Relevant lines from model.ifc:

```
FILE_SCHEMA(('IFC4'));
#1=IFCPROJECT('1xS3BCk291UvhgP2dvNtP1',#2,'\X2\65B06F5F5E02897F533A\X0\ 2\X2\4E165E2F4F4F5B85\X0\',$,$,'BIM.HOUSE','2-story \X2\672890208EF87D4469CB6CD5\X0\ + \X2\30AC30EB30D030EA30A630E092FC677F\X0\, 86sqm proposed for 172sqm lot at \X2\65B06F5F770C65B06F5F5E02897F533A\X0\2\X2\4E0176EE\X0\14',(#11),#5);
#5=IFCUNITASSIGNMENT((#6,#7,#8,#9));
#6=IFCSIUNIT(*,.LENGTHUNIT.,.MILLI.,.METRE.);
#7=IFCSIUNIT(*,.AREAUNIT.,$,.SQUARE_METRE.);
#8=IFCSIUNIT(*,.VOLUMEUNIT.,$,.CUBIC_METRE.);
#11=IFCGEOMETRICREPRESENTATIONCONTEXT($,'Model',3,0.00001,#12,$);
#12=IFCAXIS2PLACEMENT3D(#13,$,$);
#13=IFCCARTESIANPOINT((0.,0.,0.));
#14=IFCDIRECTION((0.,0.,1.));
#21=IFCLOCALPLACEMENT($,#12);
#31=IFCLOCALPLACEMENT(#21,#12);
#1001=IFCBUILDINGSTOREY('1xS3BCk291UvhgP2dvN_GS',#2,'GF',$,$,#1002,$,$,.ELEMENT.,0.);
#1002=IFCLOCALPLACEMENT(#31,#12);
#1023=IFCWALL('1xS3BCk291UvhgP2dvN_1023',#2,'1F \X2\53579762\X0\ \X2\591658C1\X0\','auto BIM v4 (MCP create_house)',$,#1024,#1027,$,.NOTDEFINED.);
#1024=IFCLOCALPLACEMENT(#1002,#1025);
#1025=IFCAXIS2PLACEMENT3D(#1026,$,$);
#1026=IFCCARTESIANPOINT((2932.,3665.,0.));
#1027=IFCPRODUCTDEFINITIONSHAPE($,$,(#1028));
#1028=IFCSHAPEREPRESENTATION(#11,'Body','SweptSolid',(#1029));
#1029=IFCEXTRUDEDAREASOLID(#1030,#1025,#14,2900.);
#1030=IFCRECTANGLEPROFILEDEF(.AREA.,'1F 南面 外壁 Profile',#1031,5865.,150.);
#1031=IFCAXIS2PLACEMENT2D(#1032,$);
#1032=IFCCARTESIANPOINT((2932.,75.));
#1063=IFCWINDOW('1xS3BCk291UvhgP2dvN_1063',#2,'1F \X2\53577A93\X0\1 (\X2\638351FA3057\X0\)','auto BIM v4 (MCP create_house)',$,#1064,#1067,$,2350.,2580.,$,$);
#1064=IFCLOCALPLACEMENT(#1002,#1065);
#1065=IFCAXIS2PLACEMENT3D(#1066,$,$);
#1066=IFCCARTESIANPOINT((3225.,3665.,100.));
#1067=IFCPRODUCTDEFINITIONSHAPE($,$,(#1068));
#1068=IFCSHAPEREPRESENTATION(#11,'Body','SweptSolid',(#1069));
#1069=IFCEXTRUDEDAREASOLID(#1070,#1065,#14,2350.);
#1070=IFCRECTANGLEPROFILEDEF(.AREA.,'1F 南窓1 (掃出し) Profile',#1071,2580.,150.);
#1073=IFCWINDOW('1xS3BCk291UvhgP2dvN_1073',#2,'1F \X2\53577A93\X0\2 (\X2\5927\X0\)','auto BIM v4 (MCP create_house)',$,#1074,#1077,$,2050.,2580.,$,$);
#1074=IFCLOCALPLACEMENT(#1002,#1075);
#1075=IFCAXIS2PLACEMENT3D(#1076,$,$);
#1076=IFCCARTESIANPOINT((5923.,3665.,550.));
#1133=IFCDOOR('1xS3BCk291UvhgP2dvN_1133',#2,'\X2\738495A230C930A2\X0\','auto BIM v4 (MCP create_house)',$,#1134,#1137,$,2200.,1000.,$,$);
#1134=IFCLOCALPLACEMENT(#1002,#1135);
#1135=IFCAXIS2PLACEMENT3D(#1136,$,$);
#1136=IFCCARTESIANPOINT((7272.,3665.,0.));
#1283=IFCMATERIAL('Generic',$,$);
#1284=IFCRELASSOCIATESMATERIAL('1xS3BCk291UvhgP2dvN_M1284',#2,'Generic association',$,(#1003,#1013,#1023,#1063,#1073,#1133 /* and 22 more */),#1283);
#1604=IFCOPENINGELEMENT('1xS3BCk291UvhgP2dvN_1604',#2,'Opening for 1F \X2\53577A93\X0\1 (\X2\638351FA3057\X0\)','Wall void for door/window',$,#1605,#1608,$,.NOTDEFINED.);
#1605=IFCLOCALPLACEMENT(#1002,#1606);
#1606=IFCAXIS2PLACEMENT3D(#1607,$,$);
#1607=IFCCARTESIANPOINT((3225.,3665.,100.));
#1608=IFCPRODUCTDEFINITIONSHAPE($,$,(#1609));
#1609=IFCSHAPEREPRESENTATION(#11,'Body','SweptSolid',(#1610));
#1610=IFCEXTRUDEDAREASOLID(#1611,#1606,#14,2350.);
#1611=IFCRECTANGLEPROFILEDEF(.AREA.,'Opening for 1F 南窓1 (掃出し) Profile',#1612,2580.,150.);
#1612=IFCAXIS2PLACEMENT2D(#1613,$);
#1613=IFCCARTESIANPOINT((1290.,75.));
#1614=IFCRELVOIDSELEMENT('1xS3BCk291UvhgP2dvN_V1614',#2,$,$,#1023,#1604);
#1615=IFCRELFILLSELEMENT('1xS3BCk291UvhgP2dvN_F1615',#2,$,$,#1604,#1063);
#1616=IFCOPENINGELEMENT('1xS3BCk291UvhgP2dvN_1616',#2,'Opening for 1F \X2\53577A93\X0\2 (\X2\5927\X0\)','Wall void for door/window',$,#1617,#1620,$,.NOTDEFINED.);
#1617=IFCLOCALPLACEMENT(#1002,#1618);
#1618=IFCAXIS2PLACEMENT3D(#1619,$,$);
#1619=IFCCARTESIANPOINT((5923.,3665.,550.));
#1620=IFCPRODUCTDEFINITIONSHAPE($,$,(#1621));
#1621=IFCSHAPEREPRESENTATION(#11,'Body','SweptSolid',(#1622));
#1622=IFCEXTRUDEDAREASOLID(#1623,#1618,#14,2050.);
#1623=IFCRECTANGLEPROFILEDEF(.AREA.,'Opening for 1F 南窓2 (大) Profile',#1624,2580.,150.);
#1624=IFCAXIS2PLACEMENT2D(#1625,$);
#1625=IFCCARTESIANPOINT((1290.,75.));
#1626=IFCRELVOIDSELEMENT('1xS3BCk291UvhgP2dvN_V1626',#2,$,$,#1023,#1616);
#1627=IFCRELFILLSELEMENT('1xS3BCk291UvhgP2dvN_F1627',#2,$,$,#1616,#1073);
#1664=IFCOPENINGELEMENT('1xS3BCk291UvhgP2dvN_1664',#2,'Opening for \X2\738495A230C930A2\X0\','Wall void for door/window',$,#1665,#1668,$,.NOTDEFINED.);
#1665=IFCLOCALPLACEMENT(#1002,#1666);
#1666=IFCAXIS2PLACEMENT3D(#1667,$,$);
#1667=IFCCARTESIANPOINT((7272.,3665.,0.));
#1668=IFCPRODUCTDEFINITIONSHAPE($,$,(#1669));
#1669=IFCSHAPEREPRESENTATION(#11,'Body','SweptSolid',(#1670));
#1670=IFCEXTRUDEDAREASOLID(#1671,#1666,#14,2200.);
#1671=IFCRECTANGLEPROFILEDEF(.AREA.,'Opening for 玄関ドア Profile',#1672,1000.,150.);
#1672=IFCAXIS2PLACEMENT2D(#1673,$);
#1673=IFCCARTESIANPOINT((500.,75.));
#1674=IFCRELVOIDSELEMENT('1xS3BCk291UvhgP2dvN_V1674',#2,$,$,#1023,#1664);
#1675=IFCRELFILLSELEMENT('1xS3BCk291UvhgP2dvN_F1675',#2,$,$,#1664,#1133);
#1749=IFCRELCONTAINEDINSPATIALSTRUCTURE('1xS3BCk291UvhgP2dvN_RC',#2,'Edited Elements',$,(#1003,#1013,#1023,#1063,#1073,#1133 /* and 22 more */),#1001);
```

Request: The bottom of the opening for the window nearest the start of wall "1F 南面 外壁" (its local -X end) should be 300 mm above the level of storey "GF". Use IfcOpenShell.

```python
import numpy as np
import ifcopenshell
import ifcopenshell.api.geometry
import ifcopenshell.geom
import ifcopenshell.util.element
import ifcopenshell.util.placement
import ifcopenshell.util.shape
import ifcopenshell.util.unit

model = ifcopenshell.open("model.ifc")
unit_scale = ifcopenshell.util.unit.calculate_unit_scale(model)

window = model.by_guid("1xS3BCk291UvhgP2dvN_1063")
opening = window.FillsVoids[0].RelatingOpeningElement
storey = ifcopenshell.util.element.get_container(window, ifc_class="IfcBuildingStorey")
level = ifcopenshell.util.placement.get_local_placement(storey.ObjectPlacement)[2, 3]

# The opening's origin need not be at the sill, so measure its lowest point.
shape = ifcopenshell.geom.create_shape(ifcopenshell.geom.settings(), opening)
bottom = ifcopenshell.util.shape.get_shape_bottom_elevation(shape, shape.geometry) / unit_scale
dz = level + 300.0 - bottom

shift = np.array([0.0, 0.0, dz])
# The window is not placed relative to its opening, so move both.
for product in (opening, window):
    matrix = ifcopenshell.util.placement.get_local_placement(product.ObjectPlacement)
    matrix[:3, 3] += shift
    ifcopenshell.api.geometry.edit_object_placement(model, product=product, matrix=matrix, is_si=False)

print(f"moved by {dz * unit_scale:+.3f} m")

model.write("model_v2.ifc")
```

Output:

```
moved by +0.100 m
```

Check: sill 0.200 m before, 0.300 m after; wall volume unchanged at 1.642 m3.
